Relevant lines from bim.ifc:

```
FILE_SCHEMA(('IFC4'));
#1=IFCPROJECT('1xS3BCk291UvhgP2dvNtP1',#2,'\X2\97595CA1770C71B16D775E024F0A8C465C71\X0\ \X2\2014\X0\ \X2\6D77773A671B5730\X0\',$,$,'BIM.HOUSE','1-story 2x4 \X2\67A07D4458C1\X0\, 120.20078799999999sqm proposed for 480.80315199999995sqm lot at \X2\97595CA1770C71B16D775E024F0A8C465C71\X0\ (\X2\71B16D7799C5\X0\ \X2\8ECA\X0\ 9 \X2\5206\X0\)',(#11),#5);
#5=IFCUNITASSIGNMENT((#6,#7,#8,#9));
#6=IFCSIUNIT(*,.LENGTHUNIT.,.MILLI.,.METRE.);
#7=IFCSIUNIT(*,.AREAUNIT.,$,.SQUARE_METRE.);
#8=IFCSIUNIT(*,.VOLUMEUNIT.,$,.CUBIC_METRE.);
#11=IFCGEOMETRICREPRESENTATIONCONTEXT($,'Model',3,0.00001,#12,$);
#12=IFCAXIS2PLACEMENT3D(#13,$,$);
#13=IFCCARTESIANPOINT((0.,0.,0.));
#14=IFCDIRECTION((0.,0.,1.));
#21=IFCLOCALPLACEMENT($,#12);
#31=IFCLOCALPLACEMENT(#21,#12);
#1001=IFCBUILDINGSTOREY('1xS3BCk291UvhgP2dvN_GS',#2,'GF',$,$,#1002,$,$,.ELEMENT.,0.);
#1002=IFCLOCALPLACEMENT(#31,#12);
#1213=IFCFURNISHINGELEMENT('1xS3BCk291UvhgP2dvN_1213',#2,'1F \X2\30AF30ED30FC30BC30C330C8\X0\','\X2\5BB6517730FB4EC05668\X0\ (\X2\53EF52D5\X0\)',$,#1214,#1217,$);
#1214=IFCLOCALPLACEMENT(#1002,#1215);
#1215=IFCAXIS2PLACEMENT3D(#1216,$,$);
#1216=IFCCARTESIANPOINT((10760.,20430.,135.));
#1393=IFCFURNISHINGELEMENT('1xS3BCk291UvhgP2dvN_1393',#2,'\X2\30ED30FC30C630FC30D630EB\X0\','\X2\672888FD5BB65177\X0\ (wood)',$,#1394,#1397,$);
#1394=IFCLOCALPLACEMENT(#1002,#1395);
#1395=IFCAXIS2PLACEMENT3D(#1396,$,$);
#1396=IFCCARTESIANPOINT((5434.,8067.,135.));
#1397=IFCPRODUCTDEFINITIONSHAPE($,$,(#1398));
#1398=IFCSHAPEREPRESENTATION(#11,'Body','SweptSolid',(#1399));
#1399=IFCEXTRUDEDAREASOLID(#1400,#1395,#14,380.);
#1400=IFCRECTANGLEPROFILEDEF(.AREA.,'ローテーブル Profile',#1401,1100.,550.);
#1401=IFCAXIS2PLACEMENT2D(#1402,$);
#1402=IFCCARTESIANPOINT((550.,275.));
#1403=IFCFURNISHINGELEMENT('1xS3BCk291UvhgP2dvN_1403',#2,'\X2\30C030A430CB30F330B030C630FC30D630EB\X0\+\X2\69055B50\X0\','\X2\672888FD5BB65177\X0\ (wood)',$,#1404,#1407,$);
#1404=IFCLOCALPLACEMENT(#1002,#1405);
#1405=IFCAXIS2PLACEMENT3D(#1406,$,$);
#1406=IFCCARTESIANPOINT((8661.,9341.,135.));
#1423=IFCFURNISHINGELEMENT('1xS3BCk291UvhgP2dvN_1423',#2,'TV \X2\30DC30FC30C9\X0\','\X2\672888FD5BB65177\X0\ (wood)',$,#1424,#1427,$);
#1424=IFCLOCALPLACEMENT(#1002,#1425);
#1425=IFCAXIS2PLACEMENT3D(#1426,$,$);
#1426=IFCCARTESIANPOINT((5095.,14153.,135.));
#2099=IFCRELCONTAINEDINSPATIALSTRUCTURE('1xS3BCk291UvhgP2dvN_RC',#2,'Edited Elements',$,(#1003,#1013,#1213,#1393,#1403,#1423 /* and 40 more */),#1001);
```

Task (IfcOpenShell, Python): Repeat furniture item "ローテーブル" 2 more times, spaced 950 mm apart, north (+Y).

```python
import numpy as np
import ifcopenshell
import ifcopenshell.api.geometry
import ifcopenshell.api.root
import ifcopenshell.util.element
import ifcopenshell.util.placement
import ifcopenshell.util.unit

model = ifcopenshell.open("bim.ifc")
unit_scale = ifcopenshell.util.unit.calculate_unit_scale(model)


def reuse_history(source, copy):
    """copy_class also copies each property set's owner history, people and application; keep the originals."""
    for rel in copy.IsDefinedBy:
        if rel.is_a("IfcRelDefinesByProperties") and (history := rel.RelatingPropertyDefinition.OwnerHistory):
            rel.RelatingPropertyDefinition.OwnerHistory = source.OwnerHistory
            ifcopenshell.util.element.remove_deep2(model, history)


source = model.by_guid("1xS3BCk291UvhgP2dvN_1393")
base = ifcopenshell.util.placement.get_local_placement(source.ObjectPlacement)
step = np.array([0.0, 1.0, 0.0]) * 0.95 / unit_scale

for i in range(1, 3):
    copy = ifcopenshell.api.root.copy_class(model, product=source)
    copy.Representation = ifcopenshell.util.element.copy_deep(
        model, source.Representation, exclude=["IfcGeometricRepresentationContext", "IfcRepresentationMap"]
    )
    reuse_history(source, copy)
    matrix = base.copy()
    matrix[:3, 3] += i * step
    print("added at", matrix[:3, 3].round(3) + 0.0)
    ifcopenshell.api.geometry.edit_object_placement(model, product=copy, matrix=matrix, is_si=False)

model.write("bim_v2.ifc")
```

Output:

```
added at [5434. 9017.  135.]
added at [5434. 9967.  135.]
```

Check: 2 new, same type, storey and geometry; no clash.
